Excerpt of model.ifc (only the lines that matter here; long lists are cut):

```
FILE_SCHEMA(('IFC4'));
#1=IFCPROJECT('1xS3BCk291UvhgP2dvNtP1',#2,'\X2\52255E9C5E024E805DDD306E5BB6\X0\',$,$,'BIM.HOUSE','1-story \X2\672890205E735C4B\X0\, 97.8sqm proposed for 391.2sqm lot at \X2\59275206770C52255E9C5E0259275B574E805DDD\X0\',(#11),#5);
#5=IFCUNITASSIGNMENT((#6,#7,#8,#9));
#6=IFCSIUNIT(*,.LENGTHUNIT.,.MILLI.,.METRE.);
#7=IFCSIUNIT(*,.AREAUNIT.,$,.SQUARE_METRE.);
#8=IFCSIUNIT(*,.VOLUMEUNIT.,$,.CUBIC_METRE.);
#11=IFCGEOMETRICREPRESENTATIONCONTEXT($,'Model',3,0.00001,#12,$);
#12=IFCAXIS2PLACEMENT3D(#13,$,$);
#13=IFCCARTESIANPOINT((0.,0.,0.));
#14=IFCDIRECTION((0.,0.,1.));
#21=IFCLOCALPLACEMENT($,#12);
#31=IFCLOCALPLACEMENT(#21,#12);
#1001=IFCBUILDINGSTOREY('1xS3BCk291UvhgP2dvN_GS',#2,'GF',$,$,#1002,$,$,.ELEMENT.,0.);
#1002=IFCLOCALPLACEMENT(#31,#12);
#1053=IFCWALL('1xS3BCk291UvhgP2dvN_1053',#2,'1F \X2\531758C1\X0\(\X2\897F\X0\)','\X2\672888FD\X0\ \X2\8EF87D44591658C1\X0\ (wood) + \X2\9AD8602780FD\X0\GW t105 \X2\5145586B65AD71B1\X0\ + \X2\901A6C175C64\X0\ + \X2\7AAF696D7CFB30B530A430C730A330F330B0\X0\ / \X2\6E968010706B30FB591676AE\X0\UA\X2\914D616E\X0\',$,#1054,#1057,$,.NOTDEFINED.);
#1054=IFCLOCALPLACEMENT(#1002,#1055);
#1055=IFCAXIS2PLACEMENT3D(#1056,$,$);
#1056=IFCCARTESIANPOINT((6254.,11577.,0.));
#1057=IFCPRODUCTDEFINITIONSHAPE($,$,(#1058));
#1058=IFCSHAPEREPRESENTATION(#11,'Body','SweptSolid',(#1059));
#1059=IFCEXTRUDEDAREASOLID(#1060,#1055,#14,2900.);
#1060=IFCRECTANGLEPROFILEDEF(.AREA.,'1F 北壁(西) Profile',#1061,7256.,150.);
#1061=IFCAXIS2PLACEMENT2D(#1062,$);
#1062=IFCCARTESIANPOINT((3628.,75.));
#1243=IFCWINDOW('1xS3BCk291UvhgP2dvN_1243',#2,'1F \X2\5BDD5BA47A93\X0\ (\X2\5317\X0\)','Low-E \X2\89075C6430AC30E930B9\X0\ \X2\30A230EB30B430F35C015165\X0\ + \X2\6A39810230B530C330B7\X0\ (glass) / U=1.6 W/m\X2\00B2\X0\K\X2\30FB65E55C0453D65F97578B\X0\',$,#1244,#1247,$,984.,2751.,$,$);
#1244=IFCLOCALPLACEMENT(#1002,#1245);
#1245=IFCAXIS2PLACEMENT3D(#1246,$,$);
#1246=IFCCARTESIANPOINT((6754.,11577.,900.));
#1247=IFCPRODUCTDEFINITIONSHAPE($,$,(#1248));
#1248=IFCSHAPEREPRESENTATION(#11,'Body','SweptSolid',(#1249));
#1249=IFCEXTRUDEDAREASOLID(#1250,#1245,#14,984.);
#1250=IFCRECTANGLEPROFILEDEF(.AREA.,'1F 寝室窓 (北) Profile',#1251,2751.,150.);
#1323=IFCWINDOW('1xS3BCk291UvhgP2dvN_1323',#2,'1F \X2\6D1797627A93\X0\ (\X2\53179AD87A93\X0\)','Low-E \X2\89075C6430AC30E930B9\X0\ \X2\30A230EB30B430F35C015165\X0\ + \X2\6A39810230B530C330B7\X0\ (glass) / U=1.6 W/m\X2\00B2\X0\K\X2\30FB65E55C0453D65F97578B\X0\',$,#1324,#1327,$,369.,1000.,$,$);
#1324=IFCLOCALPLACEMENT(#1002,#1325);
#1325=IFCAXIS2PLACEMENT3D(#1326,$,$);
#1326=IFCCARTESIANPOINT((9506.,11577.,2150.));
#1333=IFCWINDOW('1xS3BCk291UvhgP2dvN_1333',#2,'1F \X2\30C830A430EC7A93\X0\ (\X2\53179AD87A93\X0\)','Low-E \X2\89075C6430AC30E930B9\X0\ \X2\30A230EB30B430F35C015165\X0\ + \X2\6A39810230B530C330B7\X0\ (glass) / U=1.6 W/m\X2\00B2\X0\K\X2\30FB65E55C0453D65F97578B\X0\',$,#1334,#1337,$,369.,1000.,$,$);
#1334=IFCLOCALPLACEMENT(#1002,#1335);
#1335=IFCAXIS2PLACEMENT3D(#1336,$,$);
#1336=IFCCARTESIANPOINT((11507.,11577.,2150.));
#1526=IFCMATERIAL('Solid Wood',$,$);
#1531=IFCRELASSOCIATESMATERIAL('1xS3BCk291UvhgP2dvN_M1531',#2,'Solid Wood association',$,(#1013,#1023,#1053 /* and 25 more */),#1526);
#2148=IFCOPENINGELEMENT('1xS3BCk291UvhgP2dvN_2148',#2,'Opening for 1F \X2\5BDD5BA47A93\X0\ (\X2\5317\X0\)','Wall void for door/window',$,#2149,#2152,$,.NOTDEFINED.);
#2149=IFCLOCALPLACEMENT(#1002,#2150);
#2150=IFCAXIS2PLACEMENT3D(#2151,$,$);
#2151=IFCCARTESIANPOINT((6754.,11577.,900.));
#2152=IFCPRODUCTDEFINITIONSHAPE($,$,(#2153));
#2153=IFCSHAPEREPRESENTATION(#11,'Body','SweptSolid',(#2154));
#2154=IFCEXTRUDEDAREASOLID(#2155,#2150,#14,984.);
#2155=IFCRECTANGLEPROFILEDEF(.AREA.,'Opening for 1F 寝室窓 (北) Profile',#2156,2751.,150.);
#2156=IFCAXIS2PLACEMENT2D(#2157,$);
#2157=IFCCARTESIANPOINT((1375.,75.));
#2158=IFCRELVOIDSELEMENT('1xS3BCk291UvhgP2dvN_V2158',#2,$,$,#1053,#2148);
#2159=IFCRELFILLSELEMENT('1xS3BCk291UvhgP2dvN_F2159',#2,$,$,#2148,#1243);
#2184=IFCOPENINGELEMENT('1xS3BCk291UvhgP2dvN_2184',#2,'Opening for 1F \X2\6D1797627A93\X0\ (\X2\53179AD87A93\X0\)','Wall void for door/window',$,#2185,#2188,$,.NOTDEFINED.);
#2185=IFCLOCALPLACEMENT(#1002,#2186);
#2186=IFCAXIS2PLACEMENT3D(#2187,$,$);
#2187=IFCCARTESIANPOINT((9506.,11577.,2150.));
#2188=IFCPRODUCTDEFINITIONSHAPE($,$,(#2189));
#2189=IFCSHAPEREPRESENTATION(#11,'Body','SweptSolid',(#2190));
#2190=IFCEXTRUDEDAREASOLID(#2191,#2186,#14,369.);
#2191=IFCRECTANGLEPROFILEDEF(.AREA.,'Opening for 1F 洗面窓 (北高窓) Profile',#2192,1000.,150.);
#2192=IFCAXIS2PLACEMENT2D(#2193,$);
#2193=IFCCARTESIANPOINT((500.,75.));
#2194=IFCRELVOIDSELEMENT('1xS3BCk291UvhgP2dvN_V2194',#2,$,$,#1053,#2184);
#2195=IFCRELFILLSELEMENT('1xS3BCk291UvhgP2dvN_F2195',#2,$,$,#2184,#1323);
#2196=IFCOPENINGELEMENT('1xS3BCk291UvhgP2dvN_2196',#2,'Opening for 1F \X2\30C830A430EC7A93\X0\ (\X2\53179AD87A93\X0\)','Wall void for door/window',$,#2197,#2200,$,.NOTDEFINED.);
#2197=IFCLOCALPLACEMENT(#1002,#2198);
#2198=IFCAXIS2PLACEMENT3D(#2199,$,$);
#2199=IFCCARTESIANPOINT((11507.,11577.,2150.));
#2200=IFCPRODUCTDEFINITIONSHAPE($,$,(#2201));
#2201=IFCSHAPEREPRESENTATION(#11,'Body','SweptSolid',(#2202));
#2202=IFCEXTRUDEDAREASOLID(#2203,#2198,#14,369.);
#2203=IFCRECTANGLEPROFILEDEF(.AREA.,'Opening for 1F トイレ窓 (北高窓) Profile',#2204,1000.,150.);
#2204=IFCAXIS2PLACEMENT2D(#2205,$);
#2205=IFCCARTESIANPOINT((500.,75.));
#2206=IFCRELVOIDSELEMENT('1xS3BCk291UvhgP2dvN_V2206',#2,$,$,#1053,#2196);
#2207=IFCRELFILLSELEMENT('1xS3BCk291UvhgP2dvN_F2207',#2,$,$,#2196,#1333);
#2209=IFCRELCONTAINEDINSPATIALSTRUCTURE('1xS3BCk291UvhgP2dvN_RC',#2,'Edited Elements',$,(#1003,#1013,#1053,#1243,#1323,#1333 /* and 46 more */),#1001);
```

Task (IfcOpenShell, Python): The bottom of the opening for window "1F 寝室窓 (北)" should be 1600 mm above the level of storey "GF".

```python
import numpy as np
import ifcopenshell
import ifcopenshell.api.geometry
import ifcopenshell.geom
import ifcopenshell.util.element
import ifcopenshell.util.placement
import ifcopenshell.util.shape
import ifcopenshell.util.unit

model = ifcopenshell.open("model.ifc")
unit_scale = ifcopenshell.util.unit.calculate_unit_scale(model)

window = model.by_guid("1xS3BCk291UvhgP2dvN_1243")
opening = window.FillsVoids[0].RelatingOpeningElement
storey = ifcopenshell.util.element.get_container(window, ifc_class="IfcBuildingStorey")
level = ifcopenshell.util.placement.get_local_placement(storey.ObjectPlacement)[2, 3]

# The opening's origin need not be at the sill, so measure its lowest point.
shape = ifcopenshell.geom.create_shape(ifcopenshell.geom.settings(), opening)
bottom = ifcopenshell.util.shape.get_shape_bottom_elevation(shape, shape.geometry) / unit_scale
dz = level + 1.6 / unit_scale - bottom

shift = np.array([0.0, 0.0, dz])
# The window is not placed relative to its opening, so move both.
for product in (opening, window):
    matrix = ifcopenshell.util.placement.get_local_placement(product.ObjectPlacement)
    matrix[:3, 3] += shift
    ifcopenshell.api.geometry.edit_object_placement(model, product=product, matrix=matrix, is_si=False)

print(f"moved by {dz * unit_scale:+.3f} m")

model.write("model-out.ifc")
```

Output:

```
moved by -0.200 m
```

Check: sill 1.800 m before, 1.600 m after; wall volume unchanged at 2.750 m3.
